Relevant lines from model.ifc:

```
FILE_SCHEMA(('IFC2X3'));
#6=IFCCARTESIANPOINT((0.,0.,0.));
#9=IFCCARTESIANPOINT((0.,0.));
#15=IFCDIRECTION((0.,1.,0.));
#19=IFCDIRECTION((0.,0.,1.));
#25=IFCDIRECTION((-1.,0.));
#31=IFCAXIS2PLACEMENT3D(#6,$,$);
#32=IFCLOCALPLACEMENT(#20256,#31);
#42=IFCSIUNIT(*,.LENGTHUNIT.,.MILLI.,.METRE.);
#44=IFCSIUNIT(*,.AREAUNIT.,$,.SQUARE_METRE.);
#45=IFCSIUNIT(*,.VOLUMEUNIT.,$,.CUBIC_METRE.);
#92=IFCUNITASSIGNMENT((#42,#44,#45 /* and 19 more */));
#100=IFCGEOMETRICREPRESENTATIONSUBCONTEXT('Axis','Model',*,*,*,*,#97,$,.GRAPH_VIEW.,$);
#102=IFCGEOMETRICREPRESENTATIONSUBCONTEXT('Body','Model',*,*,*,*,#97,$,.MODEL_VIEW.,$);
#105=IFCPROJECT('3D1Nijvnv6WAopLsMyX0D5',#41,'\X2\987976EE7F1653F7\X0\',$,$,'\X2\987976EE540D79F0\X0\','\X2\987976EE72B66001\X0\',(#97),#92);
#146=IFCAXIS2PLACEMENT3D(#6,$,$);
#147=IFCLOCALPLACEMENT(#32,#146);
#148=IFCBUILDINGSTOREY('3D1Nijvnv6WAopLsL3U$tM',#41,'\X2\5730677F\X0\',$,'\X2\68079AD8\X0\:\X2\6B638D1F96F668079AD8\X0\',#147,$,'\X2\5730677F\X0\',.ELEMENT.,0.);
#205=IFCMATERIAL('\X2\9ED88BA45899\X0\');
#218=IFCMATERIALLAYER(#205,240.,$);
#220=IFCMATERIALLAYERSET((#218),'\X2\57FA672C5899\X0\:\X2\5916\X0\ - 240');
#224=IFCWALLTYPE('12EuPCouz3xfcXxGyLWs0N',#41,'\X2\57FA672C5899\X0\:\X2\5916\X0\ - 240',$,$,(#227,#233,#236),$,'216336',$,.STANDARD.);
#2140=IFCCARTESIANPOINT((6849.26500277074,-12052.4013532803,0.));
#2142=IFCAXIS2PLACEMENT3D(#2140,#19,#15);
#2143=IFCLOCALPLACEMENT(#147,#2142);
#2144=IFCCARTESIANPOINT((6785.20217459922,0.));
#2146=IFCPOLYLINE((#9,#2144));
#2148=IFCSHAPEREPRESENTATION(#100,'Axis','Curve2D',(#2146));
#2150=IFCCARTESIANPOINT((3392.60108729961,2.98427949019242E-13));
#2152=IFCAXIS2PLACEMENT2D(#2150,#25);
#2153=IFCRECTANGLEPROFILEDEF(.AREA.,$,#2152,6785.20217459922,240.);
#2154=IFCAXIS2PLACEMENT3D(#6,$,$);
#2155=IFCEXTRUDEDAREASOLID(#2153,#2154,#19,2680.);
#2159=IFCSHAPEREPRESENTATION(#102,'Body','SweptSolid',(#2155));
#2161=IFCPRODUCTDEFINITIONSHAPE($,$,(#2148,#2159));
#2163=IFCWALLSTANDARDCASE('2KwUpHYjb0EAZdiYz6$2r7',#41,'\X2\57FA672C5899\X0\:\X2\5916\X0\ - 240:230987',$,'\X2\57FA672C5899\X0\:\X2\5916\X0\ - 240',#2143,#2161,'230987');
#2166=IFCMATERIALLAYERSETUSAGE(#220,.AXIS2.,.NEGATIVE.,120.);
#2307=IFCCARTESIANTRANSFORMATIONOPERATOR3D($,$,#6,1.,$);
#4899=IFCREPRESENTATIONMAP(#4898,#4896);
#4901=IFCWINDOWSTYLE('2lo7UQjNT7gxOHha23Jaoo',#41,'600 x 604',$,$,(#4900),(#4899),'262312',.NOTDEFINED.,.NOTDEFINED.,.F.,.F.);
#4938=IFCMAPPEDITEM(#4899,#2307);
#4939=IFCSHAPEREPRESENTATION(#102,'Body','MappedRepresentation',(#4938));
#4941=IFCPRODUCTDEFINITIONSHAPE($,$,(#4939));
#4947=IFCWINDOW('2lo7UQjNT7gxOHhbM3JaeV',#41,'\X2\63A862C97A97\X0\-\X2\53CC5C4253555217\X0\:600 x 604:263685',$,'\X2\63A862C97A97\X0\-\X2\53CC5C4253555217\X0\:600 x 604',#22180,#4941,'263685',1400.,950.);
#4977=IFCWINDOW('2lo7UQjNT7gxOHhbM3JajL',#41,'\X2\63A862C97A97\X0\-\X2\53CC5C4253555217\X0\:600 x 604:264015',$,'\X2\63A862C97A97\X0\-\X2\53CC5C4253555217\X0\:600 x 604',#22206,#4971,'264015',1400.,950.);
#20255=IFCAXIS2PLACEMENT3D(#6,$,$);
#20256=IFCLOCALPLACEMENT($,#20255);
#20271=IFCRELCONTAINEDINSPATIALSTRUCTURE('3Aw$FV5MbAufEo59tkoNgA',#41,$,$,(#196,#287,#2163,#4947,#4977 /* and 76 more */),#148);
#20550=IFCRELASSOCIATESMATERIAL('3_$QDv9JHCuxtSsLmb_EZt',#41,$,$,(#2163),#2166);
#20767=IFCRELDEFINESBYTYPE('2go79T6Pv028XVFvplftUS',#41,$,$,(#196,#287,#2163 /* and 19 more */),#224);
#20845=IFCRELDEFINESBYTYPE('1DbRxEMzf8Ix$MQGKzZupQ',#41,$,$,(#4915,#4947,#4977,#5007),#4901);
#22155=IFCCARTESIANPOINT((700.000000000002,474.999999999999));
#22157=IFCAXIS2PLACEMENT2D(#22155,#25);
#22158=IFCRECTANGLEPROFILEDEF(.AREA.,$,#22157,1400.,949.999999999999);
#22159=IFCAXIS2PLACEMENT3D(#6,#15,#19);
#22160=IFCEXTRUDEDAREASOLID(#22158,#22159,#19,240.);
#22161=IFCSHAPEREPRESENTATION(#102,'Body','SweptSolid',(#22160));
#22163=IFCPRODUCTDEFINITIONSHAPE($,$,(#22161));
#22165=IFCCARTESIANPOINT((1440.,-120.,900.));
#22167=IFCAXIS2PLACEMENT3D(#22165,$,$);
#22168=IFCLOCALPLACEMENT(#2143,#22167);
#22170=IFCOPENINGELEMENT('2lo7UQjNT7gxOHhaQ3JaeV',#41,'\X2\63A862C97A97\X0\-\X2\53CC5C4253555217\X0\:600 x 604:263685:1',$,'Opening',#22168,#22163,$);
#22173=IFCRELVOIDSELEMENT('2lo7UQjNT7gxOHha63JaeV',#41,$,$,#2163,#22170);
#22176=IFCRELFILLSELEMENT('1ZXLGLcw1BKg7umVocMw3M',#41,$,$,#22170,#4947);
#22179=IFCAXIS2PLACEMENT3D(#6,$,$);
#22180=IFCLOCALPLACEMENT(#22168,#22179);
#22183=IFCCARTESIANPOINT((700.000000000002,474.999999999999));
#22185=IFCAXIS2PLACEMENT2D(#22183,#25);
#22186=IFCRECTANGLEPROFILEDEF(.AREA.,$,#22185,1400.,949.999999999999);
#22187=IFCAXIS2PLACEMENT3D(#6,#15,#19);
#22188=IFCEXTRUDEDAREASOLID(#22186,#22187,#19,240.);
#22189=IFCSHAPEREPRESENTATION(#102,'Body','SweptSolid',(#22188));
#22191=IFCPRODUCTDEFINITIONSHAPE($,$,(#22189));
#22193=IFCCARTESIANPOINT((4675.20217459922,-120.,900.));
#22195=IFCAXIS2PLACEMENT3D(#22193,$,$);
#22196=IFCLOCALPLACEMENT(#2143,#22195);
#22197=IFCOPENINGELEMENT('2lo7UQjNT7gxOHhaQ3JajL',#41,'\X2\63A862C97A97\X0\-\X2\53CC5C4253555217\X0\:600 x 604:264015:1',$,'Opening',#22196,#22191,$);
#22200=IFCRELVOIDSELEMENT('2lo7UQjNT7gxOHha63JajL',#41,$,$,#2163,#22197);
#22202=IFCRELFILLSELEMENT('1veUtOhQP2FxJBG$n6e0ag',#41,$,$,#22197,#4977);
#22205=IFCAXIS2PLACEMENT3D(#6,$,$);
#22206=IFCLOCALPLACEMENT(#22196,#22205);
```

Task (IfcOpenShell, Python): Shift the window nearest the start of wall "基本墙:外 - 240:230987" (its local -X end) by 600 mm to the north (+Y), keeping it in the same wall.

```python
import ifcopenshell
import ifcopenshell.api.geometry
import ifcopenshell.util.placement
import ifcopenshell.util.unit

model = ifcopenshell.open("model.ifc")
unit_scale = ifcopenshell.util.unit.calculate_unit_scale(model)

window = model.by_guid("2lo7UQjNT7gxOHhbM3JaeV")
opening = window.FillsVoids[0].RelatingOpeningElement
wall = opening.VoidsElements[0].RelatingBuildingElement

wall_matrix = ifcopenshell.util.placement.get_local_placement(wall.ObjectPlacement)
shift = wall_matrix[:3, 0] * 0.6 / unit_scale
before = ifcopenshell.util.placement.get_local_placement(window.ObjectPlacement)[:3, 3].copy()

# The window is placed relative to its opening, so it follows when the opening moves.
matrix = ifcopenshell.util.placement.get_local_placement(opening.ObjectPlacement)
matrix[:3, 3] += shift
ifcopenshell.api.geometry.edit_object_placement(
    model, product=opening, matrix=matrix, is_si=False, should_transform_children=True
)

after = ifcopenshell.util.placement.get_local_placement(window.ObjectPlacement)[:3, 3]
print("window moved by", (after - before).round(3) + 0.0)

model.write("model_edited.ifc")
```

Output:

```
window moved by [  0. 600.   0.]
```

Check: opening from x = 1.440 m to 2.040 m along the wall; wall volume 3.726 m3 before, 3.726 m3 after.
